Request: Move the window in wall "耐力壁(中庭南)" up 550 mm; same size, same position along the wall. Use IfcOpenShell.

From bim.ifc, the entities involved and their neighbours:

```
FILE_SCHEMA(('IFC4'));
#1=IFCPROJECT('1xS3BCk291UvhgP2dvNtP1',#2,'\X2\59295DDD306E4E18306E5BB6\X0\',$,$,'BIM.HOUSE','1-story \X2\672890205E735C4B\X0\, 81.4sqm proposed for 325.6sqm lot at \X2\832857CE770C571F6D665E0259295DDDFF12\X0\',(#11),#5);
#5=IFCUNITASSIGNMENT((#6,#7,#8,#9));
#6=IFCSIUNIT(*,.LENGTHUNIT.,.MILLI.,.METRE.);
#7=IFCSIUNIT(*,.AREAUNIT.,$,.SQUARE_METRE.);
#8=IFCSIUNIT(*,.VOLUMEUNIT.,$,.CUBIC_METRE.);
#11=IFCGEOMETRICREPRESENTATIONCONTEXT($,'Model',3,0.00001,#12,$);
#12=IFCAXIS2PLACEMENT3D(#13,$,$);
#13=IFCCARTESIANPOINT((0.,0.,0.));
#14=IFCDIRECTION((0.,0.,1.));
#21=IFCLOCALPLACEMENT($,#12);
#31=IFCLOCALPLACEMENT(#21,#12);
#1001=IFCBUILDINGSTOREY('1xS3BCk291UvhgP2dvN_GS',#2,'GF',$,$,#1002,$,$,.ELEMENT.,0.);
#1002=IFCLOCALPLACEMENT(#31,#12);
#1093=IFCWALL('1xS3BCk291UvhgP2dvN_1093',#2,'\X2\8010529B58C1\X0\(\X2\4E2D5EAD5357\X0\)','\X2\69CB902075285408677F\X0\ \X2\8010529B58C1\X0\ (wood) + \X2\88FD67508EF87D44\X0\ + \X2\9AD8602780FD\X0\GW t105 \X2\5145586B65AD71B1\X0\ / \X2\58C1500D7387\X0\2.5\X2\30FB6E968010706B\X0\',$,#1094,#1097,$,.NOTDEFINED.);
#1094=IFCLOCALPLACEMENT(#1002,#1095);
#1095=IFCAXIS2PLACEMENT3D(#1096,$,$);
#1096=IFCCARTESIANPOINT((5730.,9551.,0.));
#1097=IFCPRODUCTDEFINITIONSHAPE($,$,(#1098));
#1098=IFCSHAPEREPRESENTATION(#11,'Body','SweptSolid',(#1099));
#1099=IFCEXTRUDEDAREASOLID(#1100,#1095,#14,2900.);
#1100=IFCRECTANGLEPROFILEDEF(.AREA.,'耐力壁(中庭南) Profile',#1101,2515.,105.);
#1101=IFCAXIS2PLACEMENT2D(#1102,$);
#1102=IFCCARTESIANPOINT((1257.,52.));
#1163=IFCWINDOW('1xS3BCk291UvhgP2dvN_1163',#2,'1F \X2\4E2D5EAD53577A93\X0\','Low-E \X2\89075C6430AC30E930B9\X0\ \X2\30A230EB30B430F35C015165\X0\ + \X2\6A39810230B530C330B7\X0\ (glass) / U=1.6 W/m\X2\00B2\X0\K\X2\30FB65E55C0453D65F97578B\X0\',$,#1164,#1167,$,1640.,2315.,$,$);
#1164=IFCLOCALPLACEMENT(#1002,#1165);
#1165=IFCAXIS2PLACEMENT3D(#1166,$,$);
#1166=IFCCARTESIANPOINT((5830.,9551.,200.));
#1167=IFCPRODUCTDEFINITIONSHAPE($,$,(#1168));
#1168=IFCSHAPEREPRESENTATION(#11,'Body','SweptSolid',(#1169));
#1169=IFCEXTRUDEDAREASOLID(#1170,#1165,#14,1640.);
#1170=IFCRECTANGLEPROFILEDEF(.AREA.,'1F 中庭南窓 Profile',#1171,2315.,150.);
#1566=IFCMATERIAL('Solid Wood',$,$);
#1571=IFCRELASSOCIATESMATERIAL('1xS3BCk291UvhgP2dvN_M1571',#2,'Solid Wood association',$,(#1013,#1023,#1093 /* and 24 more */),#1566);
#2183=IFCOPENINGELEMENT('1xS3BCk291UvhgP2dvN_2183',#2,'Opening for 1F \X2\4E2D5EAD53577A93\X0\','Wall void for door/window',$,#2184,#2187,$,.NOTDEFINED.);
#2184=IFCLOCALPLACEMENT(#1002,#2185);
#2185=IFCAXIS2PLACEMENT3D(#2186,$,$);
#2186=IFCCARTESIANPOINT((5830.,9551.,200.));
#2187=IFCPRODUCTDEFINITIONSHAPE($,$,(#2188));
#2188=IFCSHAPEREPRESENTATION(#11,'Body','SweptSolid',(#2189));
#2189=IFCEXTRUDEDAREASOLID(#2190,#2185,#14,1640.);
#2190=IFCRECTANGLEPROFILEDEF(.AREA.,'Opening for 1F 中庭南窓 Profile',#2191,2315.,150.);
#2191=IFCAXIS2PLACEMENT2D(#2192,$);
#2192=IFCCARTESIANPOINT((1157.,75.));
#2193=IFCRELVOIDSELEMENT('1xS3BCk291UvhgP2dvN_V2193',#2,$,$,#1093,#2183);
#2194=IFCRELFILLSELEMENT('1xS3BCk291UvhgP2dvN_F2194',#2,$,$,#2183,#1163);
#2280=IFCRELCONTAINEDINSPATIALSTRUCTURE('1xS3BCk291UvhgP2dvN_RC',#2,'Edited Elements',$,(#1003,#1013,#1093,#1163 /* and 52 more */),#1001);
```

```python
import numpy as np
import ifcopenshell
import ifcopenshell.api.geometry
import ifcopenshell.util.placement
import ifcopenshell.util.unit

model = ifcopenshell.open("bim.ifc")
unit_scale = ifcopenshell.util.unit.calculate_unit_scale(model)

window = model.by_guid("1xS3BCk291UvhgP2dvN_1163")
opening = window.FillsVoids[0].RelatingOpeningElement
dz = 0.55 / unit_scale

shift = np.array([0.0, 0.0, dz])
# The window is not placed relative to its opening, so move both.
for product in (opening, window):
    matrix = ifcopenshell.util.placement.get_local_placement(product.ObjectPlacement)
    matrix[:3, 3] += shift
    ifcopenshell.api.geometry.edit_object_placement(model, product=product, matrix=matrix, is_si=False)

print(f"moved by {dz * unit_scale:+.3f} m")

model.write("bim_v2.ifc")
```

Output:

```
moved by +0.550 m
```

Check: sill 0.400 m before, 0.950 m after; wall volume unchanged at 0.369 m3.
